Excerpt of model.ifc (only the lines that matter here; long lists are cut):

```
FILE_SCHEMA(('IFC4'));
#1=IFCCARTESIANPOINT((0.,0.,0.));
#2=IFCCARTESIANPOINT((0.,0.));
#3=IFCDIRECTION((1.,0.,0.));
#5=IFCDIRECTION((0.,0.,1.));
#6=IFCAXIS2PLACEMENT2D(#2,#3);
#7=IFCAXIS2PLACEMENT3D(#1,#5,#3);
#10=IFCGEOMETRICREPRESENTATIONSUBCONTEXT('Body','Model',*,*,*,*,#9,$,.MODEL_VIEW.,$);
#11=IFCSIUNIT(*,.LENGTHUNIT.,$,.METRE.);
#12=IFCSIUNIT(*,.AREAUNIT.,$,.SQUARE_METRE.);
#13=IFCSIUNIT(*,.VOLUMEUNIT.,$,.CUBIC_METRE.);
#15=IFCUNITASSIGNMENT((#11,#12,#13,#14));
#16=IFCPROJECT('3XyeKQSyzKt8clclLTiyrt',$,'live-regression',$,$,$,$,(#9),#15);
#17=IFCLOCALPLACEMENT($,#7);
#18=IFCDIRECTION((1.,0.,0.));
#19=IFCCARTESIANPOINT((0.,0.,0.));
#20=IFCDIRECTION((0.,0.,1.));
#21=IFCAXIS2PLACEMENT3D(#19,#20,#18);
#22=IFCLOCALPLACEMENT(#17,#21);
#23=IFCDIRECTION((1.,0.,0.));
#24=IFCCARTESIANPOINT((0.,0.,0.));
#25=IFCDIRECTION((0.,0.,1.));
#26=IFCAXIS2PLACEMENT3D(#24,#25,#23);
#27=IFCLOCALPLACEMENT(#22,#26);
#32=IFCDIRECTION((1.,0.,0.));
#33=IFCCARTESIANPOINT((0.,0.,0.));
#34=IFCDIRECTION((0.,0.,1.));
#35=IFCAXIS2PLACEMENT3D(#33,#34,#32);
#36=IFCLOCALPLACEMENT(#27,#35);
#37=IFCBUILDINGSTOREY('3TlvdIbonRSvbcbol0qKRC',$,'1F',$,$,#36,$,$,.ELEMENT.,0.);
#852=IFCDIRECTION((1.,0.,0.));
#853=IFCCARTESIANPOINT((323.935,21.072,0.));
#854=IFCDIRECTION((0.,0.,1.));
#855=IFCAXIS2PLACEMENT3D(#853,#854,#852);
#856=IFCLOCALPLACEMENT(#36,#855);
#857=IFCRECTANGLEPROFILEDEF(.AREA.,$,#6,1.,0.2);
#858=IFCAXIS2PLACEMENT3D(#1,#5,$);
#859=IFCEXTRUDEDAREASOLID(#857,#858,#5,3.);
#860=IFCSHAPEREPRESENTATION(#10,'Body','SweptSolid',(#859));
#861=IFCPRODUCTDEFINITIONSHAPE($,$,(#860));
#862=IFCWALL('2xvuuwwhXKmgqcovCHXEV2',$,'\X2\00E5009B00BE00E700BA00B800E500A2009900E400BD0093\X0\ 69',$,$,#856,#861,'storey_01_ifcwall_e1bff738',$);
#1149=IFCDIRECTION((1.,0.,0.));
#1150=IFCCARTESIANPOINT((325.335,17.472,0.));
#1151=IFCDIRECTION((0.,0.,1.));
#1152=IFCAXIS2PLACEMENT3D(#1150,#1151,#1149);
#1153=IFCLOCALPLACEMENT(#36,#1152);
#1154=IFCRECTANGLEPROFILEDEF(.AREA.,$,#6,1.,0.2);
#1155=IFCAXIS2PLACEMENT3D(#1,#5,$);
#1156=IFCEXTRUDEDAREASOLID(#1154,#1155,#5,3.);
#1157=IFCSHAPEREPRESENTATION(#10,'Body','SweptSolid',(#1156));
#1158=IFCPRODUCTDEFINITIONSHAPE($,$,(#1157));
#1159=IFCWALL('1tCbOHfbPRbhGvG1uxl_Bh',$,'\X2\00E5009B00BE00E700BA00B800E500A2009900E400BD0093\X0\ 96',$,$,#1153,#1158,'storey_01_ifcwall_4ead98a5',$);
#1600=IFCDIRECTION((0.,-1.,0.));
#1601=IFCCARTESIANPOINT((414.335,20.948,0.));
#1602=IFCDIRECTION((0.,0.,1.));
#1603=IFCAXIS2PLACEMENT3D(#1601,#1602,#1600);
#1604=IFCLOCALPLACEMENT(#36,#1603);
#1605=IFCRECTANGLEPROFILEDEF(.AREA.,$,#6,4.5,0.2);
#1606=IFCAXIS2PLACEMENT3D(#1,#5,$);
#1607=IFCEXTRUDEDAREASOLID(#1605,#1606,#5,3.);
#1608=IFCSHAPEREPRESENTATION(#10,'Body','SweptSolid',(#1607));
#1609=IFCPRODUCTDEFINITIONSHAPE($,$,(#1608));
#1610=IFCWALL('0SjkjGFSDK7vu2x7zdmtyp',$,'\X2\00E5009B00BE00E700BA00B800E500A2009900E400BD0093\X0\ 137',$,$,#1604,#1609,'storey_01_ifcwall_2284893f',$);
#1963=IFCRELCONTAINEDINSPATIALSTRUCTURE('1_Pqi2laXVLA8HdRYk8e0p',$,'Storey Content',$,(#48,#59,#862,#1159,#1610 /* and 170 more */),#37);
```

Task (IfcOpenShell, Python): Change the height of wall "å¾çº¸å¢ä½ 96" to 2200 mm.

```python
import ifcopenshell
import ifcopenshell.geom
import ifcopenshell.util.representation
import ifcopenshell.util.shape

model = ifcopenshell.open("model.ifc")
settings = ifcopenshell.geom.settings()


def volume(element):
    """Net volume in cubic metres, openings subtracted."""
    shape = ifcopenshell.geom.create_shape(settings, element)
    return ifcopenshell.util.shape.get_volume(shape.geometry)


wall = model.by_guid("1tCbOHfbPRbhGvG1uxl_Bh")
before = volume(wall)

body = ifcopenshell.util.representation.get_representation(wall, "Model", "Body")
solid = body.Items[0]
old_height = solid.Depth
solid.Depth = 2.2
after = volume(wall)

print(f"height {old_height:g} -> {solid.Depth:g}, volume {before:.3f} -> {after:.3f} m3")

model.write("model_edited.ifc")
```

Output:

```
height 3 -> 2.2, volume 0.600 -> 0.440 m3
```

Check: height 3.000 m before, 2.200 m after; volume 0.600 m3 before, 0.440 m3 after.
